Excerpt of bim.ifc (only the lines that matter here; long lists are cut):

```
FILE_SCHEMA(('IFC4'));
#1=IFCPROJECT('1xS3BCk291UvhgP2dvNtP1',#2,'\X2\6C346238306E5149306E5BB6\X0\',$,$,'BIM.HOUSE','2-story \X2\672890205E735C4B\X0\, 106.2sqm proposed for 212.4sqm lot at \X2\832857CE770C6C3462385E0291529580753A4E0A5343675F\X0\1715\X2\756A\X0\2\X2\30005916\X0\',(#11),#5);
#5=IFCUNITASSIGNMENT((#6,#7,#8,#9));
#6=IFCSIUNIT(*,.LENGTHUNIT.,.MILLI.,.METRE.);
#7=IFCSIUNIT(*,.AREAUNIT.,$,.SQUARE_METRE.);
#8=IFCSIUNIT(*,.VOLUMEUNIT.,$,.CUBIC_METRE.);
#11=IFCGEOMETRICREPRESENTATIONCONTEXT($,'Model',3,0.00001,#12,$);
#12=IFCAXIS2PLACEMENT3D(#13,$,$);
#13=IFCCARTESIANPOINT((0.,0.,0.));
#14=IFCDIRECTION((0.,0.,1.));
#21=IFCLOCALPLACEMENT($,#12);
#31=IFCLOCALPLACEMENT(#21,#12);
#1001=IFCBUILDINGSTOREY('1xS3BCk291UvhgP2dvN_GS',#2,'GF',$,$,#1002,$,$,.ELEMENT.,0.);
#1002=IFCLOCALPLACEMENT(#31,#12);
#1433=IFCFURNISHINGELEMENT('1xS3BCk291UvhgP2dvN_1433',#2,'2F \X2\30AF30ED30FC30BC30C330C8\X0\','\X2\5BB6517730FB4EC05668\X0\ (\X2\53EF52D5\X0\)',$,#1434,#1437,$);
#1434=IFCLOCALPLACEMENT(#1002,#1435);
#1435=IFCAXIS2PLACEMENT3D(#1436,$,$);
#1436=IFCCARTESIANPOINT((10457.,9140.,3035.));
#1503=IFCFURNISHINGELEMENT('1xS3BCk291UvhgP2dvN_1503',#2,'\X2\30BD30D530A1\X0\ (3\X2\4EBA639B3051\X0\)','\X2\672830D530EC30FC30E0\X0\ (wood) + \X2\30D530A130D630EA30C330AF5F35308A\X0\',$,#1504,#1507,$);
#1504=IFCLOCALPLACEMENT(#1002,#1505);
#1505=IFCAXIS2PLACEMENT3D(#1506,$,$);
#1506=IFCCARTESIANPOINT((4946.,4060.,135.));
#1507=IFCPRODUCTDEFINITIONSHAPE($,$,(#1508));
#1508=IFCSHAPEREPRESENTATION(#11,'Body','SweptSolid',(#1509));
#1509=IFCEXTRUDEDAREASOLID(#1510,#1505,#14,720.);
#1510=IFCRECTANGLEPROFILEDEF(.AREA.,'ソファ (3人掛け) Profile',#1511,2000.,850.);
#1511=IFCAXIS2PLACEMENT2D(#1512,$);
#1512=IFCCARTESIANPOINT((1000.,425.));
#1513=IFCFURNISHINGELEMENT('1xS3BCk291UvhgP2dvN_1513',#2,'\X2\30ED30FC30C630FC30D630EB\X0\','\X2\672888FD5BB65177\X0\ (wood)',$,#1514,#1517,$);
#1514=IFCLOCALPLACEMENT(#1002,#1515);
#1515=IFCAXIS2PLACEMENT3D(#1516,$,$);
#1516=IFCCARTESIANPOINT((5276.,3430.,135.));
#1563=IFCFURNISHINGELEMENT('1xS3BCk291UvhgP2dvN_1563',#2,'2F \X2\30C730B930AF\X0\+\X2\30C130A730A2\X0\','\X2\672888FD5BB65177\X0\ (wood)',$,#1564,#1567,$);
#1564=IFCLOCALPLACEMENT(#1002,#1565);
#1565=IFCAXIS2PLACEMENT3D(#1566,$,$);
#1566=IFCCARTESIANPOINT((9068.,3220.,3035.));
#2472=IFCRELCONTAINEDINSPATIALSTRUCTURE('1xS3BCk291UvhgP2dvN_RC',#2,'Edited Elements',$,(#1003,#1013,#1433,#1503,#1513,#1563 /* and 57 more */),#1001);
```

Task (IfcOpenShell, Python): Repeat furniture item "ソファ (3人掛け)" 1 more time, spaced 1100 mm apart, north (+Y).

```python
import numpy as np
import ifcopenshell
import ifcopenshell.api.geometry
import ifcopenshell.api.root
import ifcopenshell.util.element
import ifcopenshell.util.placement
import ifcopenshell.util.unit

model = ifcopenshell.open("bim.ifc")
unit_scale = ifcopenshell.util.unit.calculate_unit_scale(model)


def reuse_history(source, copy):
    """copy_class also copies each property set's owner history, people and application; keep the originals."""
    for rel in copy.IsDefinedBy:
        if rel.is_a("IfcRelDefinesByProperties") and (history := rel.RelatingPropertyDefinition.OwnerHistory):
            rel.RelatingPropertyDefinition.OwnerHistory = source.OwnerHistory
            ifcopenshell.util.element.remove_deep2(model, history)


source = model.by_id(1503)
base = ifcopenshell.util.placement.get_local_placement(source.ObjectPlacement)
step = np.array([0.0, 1.0, 0.0]) * 1.1 / unit_scale

for i in range(1, 2):
    copy = ifcopenshell.api.root.copy_class(model, product=source)
    copy.Representation = ifcopenshell.util.element.copy_deep(
        model, source.Representation, exclude=["IfcGeometricRepresentationContext", "IfcRepresentationMap"]
    )
    reuse_history(source, copy)
    matrix = base.copy()
    matrix[:3, 3] += i * step
    print("added at", matrix[:3, 3].round(3) + 0.0)
    ifcopenshell.api.geometry.edit_object_placement(model, product=copy, matrix=matrix, is_si=False)

model.write("bim_updated.ifc")
```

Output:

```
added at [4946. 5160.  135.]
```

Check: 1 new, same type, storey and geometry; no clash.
